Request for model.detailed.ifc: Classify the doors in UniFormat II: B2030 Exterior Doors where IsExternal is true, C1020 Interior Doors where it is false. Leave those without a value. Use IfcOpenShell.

First a look at what the model holds.

```python
import ifcopenshell
import ifcopenshell.util.element

model = ifcopenshell.open("model.detailed.ifc")
print(model.schema)
print("classifications:", [c.Name for c in model.by_type("IfcClassification")])
values = [ifcopenshell.util.element.get_pset(e, "Pset_DoorCommon", "IsExternal") for e in model.by_type("IfcDoor")]
for value in (True, False, None):
    print("IsExternal", value, values.count(value))
```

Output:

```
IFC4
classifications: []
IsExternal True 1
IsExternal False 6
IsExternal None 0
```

```python
import ifcopenshell
import ifcopenshell.api.classification
import ifcopenshell.util.element

model = ifcopenshell.open("model.detailed.ifc")

system = ifcopenshell.api.classification.add_classification(model, classification="UniFormat II")

doors = model.by_type("IfcDoor")
external = {e: ifcopenshell.util.element.get_pset(e, "Pset_DoorCommon", "IsExternal") for e in doors}
for flag, code, name in ((True, "B2030", "Exterior Doors"), (False, "C1020", "Interior Doors")):
    products = [e for e in doors if external[e] is flag]
    ifcopenshell.api.classification.add_reference(
        model, products=products, classification=system, identification=code, name=name
    )
    print(code, len(products))

model.write("model.detailed-out.ifc")
```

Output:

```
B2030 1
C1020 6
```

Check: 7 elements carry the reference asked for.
